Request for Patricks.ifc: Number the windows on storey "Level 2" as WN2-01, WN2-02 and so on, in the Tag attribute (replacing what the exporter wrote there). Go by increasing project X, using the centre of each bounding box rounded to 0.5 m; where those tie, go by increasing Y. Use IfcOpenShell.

First a look at what the model holds.

```python
import ifcopenshell
import ifcopenshell.util.element
import ifcopenshell.util.placement

model = ifcopenshell.open("Patricks.ifc")
print(model.schema)
storey = next(s for s in model.by_type("IfcBuildingStorey") if s.Name == "Level 2")
windows = [e for e in ifcopenshell.util.element.get_decomposition(storey) if e.is_a("IfcWindow")]
for e in sorted(windows, key=lambda e: e.id()):
    origin = ifcopenshell.util.placement.get_local_placement(e.ObjectPlacement)[:3, 3]
    print(e.id(), e.Tag, e.Name, origin.round(2) + 0.0, sep=" | ")
```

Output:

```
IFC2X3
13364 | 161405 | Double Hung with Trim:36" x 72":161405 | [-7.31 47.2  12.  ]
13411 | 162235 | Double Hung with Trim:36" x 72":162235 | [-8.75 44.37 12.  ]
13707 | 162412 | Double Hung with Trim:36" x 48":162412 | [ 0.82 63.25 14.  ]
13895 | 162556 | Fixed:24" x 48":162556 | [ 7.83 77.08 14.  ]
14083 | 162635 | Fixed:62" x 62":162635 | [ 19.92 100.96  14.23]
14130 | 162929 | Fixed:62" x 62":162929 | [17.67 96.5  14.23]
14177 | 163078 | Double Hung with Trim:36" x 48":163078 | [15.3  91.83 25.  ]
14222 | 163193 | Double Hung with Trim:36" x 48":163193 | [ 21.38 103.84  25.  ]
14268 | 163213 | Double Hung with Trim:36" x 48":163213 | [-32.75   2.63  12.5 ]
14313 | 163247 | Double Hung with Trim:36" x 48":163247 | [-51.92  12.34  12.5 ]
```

```python
import ifcopenshell
import ifcopenshell.geom
import ifcopenshell.util.element
import ifcopenshell.util.shape

model = ifcopenshell.open("Patricks.ifc")
settings = ifcopenshell.geom.settings()
settings.set("use-world-coords", True)


def centre(element):
    shape = ifcopenshell.geom.create_shape(settings, element)
    return ifcopenshell.util.shape.get_bbox_centroid(shape.geometry)


storey = next(s for s in model.by_type("IfcBuildingStorey") if s.Name == "Level 2")
windows = [e for e in ifcopenshell.util.element.get_decomposition(storey) if e.is_a("IfcWindow")]

# Insertion points can sit at a corner or the storey origin, so sort by the geometry (in metres).
centres = {e: centre(e) for e in windows}
windows.sort(key=lambda e: (round(centres[e][0] / 0.5), centres[e][1]))

for i, e in enumerate(windows, start=1):
    number = f"WN2-{i:02d}"
    e.Tag = number
    print(e.id(), number)

model.write("Patricks-out.ifc")
```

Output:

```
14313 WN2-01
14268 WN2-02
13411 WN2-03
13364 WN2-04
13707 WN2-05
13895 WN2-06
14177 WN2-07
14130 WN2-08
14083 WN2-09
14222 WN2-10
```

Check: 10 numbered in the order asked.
